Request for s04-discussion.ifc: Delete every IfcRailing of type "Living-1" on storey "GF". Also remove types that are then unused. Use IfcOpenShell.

First a look at what the model holds.

```python
import ifcopenshell
import ifcopenshell.util.element

model = ifcopenshell.open("s04-discussion.ifc")
print(model.schema)
storey = next(s for s in model.by_type("IfcBuildingStorey") if s.Name == "GF")
railings = [e for e in ifcopenshell.util.element.get_decomposition(storey) if e.is_a("IfcRailing")]
seen = {}
for e in railings:
    element_type = ifcopenshell.util.element.get_type(e)
    name = element_type.Name if element_type not in (None, e) else None
    seen[name] = seen.get(name, 0) + 1
for name, count in sorted(seen.items(), key=str):
    print(count, "x", name)
```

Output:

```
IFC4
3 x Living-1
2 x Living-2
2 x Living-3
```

```python
import ifcopenshell
import ifcopenshell.api.root
import ifcopenshell.util.element

model = ifcopenshell.open("s04-discussion.ifc")

storey = next(s for s in model.by_type("IfcBuildingStorey") if s.Name == "GF")
railings = [e for e in ifcopenshell.util.element.get_decomposition(storey) if e.is_a("IfcRailing")]
targets = [e for e in railings if (t := ifcopenshell.util.element.get_type(e)) not in (None, e) and t.Name == "Living-1"]
types = {ifcopenshell.util.element.get_type(e) for e in targets} - {None, *targets}

for e in targets:
    ifcopenshell.api.root.remove_product(model, product=e)
print(len(targets), "removed")

unused = [t for t in types if not ifcopenshell.util.element.get_types(t)]
for t in unused:
    ifcopenshell.api.root.remove_product(model, product=t)
print(len(unused), "unused types removed")

model.write("s04-discussion_v2.ifc")
```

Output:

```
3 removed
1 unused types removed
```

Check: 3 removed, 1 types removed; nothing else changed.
